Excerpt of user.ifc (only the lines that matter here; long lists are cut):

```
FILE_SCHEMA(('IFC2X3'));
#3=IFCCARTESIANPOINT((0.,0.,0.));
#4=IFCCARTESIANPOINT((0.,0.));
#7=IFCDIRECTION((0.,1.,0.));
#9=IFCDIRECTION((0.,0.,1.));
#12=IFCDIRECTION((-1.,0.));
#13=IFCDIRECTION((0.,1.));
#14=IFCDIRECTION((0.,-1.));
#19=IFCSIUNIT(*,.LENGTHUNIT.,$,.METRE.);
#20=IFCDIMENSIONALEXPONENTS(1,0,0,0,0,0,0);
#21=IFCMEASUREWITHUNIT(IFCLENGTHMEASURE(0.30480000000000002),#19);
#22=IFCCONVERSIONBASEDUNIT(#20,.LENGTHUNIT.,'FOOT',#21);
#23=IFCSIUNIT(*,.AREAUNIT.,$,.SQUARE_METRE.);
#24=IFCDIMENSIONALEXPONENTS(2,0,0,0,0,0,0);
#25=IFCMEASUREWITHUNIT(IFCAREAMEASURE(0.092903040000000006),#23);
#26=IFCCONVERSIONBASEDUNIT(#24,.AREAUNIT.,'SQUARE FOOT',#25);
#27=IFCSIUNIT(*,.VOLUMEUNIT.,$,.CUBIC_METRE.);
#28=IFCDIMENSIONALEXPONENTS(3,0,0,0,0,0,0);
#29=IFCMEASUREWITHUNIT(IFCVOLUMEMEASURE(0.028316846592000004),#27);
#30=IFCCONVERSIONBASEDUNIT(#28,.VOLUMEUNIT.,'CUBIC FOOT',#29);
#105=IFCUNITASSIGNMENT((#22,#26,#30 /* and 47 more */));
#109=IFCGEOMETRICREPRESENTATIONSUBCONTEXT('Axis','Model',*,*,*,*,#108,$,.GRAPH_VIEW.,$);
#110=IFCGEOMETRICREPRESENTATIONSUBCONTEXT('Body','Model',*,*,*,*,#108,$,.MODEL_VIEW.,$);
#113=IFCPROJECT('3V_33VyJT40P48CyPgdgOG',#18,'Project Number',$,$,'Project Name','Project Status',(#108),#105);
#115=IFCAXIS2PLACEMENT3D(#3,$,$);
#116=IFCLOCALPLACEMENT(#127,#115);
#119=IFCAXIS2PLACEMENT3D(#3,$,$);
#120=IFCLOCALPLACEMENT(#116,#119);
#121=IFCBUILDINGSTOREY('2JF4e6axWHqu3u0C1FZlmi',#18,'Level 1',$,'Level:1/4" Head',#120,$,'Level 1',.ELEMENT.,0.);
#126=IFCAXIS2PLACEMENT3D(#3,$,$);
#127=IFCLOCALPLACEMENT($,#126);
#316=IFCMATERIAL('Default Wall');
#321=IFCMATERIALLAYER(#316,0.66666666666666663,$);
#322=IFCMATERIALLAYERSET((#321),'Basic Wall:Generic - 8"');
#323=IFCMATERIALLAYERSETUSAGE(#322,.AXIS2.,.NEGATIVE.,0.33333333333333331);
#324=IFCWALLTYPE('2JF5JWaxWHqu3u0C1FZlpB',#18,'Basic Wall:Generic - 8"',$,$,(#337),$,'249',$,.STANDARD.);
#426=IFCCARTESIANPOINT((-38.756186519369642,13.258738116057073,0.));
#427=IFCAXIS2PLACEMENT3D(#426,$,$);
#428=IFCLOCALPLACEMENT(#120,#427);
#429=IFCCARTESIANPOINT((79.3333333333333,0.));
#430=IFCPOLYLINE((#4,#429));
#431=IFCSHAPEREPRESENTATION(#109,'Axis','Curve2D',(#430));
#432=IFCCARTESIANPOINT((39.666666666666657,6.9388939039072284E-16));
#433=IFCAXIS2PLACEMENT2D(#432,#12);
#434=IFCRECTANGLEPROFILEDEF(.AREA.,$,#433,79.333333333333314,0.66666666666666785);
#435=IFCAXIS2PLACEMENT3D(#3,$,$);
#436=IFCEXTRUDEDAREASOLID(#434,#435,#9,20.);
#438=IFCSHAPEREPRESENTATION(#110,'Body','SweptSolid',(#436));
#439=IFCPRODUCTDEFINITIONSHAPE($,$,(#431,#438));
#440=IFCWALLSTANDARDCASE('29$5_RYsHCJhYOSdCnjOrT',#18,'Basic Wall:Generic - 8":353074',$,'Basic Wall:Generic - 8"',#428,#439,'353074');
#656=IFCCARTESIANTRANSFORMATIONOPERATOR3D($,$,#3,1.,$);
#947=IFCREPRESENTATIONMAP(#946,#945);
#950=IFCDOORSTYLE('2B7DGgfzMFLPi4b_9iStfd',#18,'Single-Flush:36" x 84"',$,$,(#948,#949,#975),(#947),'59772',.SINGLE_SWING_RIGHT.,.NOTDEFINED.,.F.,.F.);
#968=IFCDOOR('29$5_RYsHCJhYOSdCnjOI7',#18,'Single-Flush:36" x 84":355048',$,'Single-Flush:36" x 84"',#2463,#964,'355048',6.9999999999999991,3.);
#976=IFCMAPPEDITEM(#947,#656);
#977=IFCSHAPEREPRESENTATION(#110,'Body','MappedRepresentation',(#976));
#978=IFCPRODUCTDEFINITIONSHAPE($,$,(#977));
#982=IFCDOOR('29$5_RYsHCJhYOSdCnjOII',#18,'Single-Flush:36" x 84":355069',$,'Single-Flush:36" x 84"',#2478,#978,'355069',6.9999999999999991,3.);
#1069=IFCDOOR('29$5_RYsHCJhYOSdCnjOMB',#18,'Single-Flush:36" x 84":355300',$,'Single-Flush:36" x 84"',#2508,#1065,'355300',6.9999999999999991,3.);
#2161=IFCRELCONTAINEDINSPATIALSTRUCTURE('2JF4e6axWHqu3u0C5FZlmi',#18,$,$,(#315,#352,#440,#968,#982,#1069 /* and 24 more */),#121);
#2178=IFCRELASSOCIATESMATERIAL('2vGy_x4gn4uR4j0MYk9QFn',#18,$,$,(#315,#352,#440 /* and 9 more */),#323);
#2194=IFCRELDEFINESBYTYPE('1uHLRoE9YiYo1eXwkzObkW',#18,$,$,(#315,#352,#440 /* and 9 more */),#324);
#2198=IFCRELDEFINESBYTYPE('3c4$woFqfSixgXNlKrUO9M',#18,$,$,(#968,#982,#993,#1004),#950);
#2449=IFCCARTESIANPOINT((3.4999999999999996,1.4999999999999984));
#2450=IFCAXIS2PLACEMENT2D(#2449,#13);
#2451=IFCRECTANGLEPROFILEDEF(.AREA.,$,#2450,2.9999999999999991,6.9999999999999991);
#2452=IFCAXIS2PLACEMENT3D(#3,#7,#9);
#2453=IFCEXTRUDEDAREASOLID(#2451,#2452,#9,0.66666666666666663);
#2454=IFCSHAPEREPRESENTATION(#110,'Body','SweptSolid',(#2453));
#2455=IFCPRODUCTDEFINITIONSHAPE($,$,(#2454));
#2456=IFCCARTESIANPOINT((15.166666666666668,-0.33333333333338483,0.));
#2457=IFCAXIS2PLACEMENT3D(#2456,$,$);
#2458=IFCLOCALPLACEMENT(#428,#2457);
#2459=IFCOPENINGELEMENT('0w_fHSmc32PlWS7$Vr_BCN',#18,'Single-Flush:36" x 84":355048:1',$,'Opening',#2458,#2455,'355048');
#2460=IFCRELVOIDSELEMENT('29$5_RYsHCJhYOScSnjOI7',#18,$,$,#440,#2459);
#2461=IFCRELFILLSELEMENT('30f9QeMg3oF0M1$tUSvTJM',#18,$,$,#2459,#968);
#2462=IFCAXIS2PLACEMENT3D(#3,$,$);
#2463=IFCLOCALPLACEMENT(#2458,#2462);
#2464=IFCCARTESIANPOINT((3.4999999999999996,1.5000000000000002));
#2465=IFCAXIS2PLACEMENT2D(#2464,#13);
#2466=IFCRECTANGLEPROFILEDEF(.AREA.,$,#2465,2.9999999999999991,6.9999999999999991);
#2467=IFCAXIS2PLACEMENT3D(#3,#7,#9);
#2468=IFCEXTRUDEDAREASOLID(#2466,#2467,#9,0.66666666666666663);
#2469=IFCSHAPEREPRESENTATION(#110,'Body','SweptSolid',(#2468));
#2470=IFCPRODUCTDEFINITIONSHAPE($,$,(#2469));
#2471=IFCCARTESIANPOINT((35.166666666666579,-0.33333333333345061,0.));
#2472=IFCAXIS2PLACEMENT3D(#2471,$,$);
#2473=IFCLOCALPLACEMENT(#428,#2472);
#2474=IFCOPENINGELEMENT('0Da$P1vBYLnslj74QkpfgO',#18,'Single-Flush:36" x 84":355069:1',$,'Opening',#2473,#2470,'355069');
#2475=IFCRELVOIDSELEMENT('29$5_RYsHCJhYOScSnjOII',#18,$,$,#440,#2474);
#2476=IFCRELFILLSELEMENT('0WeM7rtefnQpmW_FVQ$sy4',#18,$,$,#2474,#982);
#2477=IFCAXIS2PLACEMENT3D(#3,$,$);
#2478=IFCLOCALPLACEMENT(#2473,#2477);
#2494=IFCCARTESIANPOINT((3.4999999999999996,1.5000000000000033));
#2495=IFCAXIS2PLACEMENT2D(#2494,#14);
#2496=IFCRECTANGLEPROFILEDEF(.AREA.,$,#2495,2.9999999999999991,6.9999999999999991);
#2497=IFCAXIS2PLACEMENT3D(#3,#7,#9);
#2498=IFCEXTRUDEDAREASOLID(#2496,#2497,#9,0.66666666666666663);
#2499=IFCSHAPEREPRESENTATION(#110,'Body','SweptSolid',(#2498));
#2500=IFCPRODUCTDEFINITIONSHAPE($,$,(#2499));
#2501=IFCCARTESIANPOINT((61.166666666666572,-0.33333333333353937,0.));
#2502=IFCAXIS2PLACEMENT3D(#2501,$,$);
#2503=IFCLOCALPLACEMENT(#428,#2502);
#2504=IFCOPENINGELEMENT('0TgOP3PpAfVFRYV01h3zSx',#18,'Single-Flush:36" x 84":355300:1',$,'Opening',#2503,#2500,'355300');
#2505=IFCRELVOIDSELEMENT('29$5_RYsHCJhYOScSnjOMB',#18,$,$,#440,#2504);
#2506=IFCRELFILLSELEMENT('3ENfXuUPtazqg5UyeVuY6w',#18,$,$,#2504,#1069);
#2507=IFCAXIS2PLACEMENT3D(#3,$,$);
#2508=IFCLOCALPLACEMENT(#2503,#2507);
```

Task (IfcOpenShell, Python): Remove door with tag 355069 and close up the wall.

```python
import ifcopenshell
import ifcopenshell.api.feature
import ifcopenshell.api.root
import ifcopenshell.geom
import ifcopenshell.util.shape

model = ifcopenshell.open("user.ifc")
settings = ifcopenshell.geom.settings()


def volume(element):
    """Net volume in cubic metres, openings subtracted."""
    shape = ifcopenshell.geom.create_shape(settings, element)
    return ifcopenshell.util.shape.get_volume(shape.geometry)


door = model.by_id(982)
opening = door.FillsVoids[0].RelatingOpeningElement
wall = opening.VoidsElements[0].RelatingBuildingElement
before = volume(wall)

ifcopenshell.api.root.remove_product(model, product=door)
ifcopenshell.api.feature.remove_feature(model, feature=opening)

after = volume(wall)

print(f"wall volume {before:.3f} -> {after:.3f} m3")

model.write("user_v2.ifc")
```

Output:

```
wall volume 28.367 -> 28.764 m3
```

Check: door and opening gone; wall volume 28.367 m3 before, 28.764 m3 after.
